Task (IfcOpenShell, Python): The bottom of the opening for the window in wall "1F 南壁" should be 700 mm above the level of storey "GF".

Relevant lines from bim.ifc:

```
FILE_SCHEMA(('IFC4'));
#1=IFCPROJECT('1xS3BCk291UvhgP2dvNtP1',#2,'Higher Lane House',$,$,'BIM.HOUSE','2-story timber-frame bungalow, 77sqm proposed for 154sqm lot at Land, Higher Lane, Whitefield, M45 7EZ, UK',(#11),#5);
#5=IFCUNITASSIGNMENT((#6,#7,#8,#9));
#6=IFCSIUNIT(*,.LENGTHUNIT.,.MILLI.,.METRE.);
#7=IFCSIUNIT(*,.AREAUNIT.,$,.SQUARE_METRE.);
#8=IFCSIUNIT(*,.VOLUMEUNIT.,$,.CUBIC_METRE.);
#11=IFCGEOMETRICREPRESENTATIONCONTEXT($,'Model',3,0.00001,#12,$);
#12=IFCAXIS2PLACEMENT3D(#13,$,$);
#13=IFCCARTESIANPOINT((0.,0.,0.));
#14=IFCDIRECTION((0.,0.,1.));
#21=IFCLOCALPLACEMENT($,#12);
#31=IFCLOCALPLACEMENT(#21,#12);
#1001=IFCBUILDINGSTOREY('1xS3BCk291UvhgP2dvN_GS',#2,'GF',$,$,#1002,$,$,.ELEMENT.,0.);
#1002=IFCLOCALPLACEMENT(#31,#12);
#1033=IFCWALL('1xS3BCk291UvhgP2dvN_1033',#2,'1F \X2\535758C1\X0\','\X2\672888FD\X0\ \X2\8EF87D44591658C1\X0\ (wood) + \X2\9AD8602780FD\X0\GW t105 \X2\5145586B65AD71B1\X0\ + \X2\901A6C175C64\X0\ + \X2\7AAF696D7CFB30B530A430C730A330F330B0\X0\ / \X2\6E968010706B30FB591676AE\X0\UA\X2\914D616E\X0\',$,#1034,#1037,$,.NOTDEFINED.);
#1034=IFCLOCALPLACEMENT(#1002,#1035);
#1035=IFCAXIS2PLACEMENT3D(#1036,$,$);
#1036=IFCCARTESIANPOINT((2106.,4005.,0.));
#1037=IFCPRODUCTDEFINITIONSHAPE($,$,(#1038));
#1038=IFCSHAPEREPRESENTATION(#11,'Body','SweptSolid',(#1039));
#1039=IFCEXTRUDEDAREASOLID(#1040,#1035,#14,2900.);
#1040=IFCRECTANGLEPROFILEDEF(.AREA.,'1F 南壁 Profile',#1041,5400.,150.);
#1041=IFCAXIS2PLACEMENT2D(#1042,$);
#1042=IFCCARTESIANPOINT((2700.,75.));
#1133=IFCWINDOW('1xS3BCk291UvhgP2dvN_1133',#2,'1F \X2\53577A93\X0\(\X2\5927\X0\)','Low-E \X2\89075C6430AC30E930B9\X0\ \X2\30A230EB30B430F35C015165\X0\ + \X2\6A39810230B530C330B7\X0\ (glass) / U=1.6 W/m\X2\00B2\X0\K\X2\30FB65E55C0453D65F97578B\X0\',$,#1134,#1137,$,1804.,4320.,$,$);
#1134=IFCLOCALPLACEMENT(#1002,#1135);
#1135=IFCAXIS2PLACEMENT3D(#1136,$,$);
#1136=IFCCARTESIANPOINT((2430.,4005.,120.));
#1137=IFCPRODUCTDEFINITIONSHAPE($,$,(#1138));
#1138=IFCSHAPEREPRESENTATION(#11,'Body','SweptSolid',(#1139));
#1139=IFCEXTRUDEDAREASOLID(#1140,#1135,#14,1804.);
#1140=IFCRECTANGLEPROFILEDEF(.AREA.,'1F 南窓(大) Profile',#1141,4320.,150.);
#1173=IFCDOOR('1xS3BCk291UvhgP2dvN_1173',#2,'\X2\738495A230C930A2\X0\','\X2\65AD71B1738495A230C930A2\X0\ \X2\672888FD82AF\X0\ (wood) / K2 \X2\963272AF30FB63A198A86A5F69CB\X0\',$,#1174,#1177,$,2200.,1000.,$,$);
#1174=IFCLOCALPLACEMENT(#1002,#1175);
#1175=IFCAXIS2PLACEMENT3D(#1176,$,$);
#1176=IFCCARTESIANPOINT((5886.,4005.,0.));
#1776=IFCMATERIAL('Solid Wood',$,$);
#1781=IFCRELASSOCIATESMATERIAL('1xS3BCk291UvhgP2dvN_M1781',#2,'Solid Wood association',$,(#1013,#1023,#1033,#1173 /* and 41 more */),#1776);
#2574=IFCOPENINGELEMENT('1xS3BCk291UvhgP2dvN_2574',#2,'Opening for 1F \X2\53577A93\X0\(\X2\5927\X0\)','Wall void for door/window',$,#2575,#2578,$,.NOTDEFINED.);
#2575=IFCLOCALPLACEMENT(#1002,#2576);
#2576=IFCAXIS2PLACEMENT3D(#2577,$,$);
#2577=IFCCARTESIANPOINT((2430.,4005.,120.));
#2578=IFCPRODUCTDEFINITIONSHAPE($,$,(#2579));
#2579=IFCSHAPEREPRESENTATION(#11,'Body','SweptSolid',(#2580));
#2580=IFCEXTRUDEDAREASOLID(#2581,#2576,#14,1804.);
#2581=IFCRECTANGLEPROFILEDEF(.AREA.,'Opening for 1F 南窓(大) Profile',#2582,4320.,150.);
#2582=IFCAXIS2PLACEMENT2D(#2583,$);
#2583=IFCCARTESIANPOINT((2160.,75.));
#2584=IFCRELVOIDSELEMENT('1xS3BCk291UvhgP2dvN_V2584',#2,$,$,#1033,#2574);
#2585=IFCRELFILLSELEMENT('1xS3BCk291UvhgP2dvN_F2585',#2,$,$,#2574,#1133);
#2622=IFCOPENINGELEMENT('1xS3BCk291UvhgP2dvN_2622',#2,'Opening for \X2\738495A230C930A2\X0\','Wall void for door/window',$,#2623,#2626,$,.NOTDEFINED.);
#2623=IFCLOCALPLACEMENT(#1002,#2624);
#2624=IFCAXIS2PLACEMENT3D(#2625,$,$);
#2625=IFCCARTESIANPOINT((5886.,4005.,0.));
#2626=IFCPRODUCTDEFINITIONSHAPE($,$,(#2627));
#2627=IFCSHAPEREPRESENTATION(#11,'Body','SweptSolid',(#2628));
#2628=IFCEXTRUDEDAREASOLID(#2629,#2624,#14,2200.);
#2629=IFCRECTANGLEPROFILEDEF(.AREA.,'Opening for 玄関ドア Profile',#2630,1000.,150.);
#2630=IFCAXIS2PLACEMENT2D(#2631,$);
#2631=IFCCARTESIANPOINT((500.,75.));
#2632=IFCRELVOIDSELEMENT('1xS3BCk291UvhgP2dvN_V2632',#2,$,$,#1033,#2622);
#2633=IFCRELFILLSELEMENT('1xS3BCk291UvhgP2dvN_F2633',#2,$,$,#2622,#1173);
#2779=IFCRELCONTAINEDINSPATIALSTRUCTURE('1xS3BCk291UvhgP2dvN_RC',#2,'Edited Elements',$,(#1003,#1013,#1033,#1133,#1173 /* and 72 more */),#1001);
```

```python
import numpy as np
import ifcopenshell
import ifcopenshell.api.geometry
import ifcopenshell.geom
import ifcopenshell.util.element
import ifcopenshell.util.placement
import ifcopenshell.util.shape
import ifcopenshell.util.unit

model = ifcopenshell.open("bim.ifc")
unit_scale = ifcopenshell.util.unit.calculate_unit_scale(model)

window = model.by_id(1133)
opening = window.FillsVoids[0].RelatingOpeningElement
storey = ifcopenshell.util.element.get_container(window, ifc_class="IfcBuildingStorey")
level = ifcopenshell.util.placement.get_local_placement(storey.ObjectPlacement)[2, 3]

# The opening's origin need not be at the sill, so measure its lowest point.
shape = ifcopenshell.geom.create_shape(ifcopenshell.geom.settings(), opening)
bottom = ifcopenshell.util.shape.get_shape_bottom_elevation(shape, shape.geometry) / unit_scale
dz = level + 0.7 / unit_scale - bottom

shift = np.array([0.0, 0.0, dz])
# The window is not placed relative to its opening, so move both.
for product in (opening, window):
    matrix = ifcopenshell.util.placement.get_local_placement(product.ObjectPlacement)
    matrix[:3, 3] += shift
    ifcopenshell.api.geometry.edit_object_placement(model, product=product, matrix=matrix, is_si=False)

print(f"moved by {dz * unit_scale:+.3f} m")

model.write("bim_updated.ifc")
```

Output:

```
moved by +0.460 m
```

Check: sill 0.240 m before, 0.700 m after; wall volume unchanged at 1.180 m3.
